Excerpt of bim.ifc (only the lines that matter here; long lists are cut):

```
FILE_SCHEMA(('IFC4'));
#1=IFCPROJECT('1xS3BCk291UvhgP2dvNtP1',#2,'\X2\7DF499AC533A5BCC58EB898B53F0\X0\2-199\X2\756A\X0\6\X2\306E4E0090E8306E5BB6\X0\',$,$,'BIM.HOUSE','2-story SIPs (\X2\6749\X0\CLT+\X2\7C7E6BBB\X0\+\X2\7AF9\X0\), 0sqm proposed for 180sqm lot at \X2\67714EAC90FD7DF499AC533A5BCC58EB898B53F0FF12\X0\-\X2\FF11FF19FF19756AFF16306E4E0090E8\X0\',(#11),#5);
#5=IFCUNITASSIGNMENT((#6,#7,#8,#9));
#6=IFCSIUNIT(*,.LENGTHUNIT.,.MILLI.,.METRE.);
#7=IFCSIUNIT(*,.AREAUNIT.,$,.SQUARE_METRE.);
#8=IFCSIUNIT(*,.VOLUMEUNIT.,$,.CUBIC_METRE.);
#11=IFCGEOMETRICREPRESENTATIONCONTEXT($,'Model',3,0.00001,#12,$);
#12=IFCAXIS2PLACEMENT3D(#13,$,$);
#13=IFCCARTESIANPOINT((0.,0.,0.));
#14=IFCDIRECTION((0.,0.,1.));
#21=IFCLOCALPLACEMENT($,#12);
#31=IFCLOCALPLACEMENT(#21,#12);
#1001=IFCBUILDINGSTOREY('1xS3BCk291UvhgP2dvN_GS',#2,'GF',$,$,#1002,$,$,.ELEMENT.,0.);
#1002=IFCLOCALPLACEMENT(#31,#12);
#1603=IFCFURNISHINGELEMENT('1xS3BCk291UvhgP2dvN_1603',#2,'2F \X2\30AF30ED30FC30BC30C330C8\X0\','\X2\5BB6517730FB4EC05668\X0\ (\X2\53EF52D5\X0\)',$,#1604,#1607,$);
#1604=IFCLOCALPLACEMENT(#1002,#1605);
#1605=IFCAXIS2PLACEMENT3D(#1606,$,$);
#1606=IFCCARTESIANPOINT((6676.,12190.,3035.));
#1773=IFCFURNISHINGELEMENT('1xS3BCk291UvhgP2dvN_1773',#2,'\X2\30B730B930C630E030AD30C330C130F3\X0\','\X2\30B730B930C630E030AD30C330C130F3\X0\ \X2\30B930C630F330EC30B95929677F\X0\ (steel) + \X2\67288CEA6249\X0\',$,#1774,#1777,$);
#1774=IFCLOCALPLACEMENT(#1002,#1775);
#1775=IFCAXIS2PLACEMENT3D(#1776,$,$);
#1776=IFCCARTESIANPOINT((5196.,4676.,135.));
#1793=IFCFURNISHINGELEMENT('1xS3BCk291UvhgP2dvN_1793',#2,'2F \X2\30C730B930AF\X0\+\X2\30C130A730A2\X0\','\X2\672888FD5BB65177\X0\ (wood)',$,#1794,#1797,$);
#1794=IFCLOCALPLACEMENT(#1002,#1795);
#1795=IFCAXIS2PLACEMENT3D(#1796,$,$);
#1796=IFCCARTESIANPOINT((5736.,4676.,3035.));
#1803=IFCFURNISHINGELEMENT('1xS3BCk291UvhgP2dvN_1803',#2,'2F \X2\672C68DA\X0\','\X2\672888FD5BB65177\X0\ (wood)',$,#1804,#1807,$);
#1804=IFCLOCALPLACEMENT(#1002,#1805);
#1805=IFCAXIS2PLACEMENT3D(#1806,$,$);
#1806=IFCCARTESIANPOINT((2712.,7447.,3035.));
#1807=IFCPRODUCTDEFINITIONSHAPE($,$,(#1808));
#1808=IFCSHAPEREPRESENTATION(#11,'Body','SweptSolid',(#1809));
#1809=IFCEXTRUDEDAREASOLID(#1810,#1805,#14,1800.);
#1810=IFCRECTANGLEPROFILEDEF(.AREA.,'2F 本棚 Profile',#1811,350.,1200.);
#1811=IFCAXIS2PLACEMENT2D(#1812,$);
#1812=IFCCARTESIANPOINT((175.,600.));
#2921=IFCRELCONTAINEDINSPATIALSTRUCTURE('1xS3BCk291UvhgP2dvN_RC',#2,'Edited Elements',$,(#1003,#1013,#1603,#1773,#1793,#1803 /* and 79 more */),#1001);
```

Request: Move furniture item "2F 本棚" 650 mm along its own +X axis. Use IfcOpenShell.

```python
import ifcopenshell
import ifcopenshell.api.geometry
import ifcopenshell.util.placement
import ifcopenshell.util.unit

model = ifcopenshell.open("bim.ifc")
unit_scale = ifcopenshell.util.unit.calculate_unit_scale(model)

item = model.by_guid("1xS3BCk291UvhgP2dvN_1803")
matrix = ifcopenshell.util.placement.get_local_placement(item.ObjectPlacement)
matrix[:3, 3] += matrix[:3, 0] * 0.65 / unit_scale
ifcopenshell.api.geometry.edit_object_placement(model, product=item, matrix=matrix, is_si=False)

print(ifcopenshell.util.placement.get_local_placement(item.ObjectPlacement).round(3) + 0.0)

model.write("bim_rev.ifc")
```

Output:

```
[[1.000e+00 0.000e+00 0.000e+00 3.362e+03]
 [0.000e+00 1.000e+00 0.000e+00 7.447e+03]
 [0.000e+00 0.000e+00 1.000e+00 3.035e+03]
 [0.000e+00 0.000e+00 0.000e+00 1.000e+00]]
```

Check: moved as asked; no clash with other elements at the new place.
